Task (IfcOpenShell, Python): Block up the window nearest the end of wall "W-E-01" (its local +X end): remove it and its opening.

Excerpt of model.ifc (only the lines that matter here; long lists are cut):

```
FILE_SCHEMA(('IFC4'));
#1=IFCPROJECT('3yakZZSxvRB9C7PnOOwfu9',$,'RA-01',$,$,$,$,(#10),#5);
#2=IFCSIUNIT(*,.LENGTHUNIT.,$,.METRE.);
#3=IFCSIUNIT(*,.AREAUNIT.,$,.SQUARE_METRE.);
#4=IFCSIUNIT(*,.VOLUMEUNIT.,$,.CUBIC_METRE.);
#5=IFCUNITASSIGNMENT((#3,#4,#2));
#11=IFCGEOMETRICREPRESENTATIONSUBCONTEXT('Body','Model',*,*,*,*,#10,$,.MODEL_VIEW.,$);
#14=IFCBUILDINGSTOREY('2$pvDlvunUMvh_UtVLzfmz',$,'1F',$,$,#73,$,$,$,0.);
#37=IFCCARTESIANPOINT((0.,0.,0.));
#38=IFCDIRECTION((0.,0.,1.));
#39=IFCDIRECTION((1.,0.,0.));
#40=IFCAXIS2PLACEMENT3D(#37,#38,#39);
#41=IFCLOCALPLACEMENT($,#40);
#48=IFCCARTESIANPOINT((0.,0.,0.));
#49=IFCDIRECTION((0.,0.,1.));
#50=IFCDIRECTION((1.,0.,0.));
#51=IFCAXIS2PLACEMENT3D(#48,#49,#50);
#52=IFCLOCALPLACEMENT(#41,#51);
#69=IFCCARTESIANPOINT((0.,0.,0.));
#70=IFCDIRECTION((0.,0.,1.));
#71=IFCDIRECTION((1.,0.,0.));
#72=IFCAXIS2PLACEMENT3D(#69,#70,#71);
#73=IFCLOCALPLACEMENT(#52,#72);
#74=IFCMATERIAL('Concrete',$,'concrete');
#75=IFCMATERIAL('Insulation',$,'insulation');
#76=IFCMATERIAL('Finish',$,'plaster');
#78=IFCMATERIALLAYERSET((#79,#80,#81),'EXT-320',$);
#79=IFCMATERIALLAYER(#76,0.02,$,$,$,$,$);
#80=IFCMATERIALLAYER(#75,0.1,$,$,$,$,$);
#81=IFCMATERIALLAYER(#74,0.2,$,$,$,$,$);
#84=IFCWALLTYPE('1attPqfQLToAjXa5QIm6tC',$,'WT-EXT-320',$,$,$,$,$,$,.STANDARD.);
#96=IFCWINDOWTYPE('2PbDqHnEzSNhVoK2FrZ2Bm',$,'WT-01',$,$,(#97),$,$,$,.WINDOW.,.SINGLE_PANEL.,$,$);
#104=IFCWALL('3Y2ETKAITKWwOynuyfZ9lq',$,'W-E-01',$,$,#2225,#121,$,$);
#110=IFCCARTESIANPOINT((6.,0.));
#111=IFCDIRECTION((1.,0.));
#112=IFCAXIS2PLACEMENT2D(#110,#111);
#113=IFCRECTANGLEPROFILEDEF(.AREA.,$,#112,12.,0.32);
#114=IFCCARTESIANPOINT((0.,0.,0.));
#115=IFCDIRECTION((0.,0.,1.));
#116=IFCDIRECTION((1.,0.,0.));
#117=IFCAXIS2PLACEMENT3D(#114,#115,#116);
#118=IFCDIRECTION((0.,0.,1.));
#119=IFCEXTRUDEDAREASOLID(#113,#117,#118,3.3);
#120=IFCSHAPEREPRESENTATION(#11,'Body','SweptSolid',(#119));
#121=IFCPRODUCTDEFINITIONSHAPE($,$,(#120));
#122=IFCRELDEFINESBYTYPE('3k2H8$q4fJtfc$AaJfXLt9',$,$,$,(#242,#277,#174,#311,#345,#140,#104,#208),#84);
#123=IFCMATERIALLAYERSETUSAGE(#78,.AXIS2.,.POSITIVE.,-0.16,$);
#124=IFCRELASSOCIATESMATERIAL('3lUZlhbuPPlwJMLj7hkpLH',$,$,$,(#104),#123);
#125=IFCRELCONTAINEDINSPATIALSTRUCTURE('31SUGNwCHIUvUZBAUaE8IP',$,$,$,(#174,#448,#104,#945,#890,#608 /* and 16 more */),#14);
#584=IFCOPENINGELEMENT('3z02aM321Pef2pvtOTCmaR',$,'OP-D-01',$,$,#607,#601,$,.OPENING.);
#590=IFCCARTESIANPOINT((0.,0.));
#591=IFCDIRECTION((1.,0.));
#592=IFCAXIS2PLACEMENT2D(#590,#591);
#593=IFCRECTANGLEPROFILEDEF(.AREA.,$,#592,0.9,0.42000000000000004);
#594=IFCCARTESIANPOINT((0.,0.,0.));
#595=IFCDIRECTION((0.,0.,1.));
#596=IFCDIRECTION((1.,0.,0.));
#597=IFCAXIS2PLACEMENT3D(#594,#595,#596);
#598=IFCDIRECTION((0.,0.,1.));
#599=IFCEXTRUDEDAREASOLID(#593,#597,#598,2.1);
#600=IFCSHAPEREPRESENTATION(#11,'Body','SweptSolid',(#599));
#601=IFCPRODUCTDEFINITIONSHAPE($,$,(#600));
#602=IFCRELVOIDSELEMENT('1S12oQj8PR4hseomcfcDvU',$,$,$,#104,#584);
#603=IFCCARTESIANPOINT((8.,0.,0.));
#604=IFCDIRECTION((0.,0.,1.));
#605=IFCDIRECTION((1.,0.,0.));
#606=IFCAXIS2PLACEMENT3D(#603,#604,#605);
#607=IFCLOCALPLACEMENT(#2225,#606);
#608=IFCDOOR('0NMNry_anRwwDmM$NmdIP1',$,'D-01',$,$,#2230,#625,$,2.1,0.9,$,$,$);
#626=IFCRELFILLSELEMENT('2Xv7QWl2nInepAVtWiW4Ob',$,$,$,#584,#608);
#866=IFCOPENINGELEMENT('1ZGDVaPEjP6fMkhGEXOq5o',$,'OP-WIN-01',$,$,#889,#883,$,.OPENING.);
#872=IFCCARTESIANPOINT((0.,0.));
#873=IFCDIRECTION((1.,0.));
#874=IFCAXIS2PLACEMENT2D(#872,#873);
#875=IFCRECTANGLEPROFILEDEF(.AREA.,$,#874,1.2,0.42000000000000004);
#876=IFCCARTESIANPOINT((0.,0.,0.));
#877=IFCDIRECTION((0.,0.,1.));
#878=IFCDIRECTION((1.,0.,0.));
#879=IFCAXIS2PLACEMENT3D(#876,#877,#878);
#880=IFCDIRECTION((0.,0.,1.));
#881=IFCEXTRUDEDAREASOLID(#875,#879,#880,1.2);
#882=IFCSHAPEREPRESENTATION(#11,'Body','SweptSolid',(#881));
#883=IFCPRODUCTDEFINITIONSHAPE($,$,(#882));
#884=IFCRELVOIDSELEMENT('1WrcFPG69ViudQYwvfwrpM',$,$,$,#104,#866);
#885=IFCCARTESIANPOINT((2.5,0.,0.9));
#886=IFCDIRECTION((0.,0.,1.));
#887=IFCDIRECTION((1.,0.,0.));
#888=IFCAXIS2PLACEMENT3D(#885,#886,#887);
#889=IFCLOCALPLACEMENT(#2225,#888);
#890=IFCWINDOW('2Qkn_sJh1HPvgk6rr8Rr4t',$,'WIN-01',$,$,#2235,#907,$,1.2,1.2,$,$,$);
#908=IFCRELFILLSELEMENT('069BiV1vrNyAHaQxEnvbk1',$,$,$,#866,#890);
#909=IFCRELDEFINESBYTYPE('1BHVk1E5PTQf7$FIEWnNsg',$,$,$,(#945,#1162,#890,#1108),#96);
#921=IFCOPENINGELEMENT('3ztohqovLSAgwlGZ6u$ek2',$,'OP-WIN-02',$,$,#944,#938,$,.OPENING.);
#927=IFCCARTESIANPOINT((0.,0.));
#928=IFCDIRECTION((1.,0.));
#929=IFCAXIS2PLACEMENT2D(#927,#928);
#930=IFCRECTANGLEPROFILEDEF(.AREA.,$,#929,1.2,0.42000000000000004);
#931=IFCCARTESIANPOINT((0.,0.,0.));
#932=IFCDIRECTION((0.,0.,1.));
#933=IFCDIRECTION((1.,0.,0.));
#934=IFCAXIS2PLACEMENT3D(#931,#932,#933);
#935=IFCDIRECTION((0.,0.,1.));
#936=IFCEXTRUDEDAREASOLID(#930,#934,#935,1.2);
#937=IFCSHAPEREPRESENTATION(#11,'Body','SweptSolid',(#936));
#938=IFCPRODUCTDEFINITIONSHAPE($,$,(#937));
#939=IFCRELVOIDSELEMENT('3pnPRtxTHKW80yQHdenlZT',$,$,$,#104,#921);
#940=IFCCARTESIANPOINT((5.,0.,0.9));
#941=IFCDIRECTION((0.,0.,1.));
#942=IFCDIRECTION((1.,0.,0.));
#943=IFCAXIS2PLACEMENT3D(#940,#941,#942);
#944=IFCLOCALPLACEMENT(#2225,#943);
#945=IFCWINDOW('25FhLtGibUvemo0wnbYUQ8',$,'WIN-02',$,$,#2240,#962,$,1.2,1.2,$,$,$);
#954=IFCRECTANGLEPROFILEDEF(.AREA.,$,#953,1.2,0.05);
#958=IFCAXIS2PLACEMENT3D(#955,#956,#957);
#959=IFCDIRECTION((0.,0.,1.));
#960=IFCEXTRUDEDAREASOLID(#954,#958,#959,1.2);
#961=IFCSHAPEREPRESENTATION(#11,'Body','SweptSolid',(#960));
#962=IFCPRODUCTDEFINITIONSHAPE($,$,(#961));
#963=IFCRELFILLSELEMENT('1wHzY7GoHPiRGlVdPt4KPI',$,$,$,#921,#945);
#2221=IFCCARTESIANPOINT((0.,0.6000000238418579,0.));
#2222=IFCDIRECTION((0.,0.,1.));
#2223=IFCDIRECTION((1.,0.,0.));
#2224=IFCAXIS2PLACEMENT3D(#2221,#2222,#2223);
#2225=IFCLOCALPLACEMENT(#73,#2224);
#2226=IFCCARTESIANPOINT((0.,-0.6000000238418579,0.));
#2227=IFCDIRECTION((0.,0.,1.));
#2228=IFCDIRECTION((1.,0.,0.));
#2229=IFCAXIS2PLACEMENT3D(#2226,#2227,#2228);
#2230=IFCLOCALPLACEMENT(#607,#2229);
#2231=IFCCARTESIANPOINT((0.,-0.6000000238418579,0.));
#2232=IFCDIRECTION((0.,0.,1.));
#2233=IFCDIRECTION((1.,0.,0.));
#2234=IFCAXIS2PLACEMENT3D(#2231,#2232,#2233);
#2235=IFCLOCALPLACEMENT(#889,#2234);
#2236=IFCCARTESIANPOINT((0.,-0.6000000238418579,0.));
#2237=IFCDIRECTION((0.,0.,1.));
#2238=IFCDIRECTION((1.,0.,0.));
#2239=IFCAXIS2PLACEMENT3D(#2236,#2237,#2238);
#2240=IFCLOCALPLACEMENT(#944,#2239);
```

```python
import ifcopenshell
import ifcopenshell.api.feature
import ifcopenshell.api.root
import ifcopenshell.geom
import ifcopenshell.util.shape

model = ifcopenshell.open("model.ifc")
settings = ifcopenshell.geom.settings()


def volume(element):
    """Net volume in cubic metres, openings subtracted."""
    shape = ifcopenshell.geom.create_shape(settings, element)
    return ifcopenshell.util.shape.get_volume(shape.geometry)


window = model.by_guid("25FhLtGibUvemo0wnbYUQ8")
opening = window.FillsVoids[0].RelatingOpeningElement
wall = opening.VoidsElements[0].RelatingBuildingElement
before = volume(wall)

ifcopenshell.api.root.remove_product(model, product=window)
ifcopenshell.api.feature.remove_feature(model, feature=opening)

after = volume(wall)

print(f"wall volume {before:.3f} -> {after:.3f} m3")

model.write("model_v2.ifc")
```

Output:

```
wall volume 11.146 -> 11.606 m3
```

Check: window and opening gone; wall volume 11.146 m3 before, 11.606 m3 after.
